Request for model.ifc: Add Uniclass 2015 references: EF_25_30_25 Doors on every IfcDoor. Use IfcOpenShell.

First a look at what the model holds.

```python
import ifcopenshell

model = ifcopenshell.open("model.ifc")
print(model.schema)
print("classifications:", [c.Name for c in model.by_type("IfcClassification")])
for ifc_class in ("IfcDoor", "IfcRoof", "IfcStair", "IfcWall", "IfcWindow"):
    print(ifc_class, len(model.by_type(ifc_class)))
```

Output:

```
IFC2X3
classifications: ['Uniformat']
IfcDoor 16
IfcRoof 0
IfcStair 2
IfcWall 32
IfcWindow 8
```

```python
import ifcopenshell
import ifcopenshell.api.classification

model = ifcopenshell.open("model.ifc")

# IFC2X3 requires Source and Edition and has no link from the project to the system.
system = model.create_entity("IfcClassification", Source="NBS", Edition="2015", Name="Uniclass 2015")

codes = {
    "IfcDoor": ("EF_25_30_25", "Doors"),
}
for ifc_class, (code, name) in codes.items():
    products = model.by_type(ifc_class)
    ifcopenshell.api.classification.add_reference(
        model, products=products, classification=system, identification=code, name=name
    )
    print(code, len(products))

model.write("model_edited.ifc")
```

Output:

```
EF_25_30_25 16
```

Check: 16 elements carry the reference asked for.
